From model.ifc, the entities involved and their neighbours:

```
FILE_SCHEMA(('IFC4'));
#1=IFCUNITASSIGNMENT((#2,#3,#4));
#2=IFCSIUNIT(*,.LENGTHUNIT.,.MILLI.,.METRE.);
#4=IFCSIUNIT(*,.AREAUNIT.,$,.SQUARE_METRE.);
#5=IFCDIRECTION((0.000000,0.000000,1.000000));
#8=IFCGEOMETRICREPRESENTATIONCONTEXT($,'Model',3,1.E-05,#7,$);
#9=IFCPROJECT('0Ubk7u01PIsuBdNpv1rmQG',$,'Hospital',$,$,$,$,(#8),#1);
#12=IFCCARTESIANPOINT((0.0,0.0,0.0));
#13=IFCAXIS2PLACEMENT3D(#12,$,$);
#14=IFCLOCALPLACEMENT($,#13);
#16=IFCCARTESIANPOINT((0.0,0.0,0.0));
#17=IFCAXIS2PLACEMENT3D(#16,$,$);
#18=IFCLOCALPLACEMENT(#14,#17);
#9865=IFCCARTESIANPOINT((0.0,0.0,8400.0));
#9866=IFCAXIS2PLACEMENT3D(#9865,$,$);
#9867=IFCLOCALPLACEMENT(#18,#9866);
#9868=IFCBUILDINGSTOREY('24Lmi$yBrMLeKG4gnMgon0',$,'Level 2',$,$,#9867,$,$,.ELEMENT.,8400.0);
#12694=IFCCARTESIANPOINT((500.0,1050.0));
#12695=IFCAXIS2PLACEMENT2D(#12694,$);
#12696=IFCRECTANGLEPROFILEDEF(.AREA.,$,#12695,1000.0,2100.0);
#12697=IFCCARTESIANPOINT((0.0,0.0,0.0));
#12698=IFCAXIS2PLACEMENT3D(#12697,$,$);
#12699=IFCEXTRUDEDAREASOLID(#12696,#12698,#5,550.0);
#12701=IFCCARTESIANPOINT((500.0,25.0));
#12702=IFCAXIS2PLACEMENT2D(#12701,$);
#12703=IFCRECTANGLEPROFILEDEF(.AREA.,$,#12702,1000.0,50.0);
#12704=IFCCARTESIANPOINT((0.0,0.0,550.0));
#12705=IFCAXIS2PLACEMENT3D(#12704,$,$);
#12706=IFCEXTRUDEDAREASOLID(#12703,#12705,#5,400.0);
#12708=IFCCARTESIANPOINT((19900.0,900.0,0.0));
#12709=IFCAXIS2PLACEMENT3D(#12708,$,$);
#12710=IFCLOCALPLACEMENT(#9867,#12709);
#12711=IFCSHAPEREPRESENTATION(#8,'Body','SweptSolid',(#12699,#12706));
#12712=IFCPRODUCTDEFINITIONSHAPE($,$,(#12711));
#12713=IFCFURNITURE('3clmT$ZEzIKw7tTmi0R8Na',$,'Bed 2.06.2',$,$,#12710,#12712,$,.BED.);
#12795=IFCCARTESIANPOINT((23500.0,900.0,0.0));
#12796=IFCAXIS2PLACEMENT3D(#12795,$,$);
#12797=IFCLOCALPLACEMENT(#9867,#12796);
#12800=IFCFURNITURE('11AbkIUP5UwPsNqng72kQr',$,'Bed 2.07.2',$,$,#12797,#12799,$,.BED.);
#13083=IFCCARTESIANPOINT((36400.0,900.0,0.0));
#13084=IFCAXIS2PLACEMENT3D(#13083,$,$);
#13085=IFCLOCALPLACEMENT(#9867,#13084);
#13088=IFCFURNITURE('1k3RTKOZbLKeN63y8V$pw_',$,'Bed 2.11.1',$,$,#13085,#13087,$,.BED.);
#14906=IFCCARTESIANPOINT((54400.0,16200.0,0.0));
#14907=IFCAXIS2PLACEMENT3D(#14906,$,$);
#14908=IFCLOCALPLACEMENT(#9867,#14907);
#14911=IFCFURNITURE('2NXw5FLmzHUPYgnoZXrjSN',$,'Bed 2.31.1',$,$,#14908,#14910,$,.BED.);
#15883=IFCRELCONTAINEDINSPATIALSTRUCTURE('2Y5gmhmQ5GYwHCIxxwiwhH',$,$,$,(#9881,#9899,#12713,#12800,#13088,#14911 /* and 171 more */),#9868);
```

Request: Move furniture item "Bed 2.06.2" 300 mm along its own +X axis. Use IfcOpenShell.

```python
import ifcopenshell
import ifcopenshell.api.geometry
import ifcopenshell.util.placement

model = ifcopenshell.open("model.ifc")

item = model.by_guid("3clmT$ZEzIKw7tTmi0R8Na")
matrix = ifcopenshell.util.placement.get_local_placement(item.ObjectPlacement)
matrix[:3, 3] += matrix[:3, 0] * 300.0
ifcopenshell.api.geometry.edit_object_placement(model, product=item, matrix=matrix, is_si=False)

print(ifcopenshell.util.placement.get_local_placement(item.ObjectPlacement).round(3) + 0.0)

model.write("model_edited.ifc")
```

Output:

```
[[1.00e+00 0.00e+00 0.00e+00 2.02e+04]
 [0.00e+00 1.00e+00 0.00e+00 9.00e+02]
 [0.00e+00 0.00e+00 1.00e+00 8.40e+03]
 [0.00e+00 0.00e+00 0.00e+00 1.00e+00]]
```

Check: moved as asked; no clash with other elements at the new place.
